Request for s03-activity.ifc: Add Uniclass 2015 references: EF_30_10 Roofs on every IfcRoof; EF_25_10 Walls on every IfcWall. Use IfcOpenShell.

First a look at what the model holds.

```python
import ifcopenshell

model = ifcopenshell.open("s03-activity.ifc")
print(model.schema)
print("classifications:", [c.Name for c in model.by_type("IfcClassification")])
for ifc_class in ("IfcDoor", "IfcRoof", "IfcStair", "IfcWall", "IfcWindow"):
    print(ifc_class, len(model.by_type(ifc_class)))
```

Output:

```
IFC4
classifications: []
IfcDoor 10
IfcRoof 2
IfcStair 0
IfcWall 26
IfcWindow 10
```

```python
import ifcopenshell
import ifcopenshell.api.classification

model = ifcopenshell.open("s03-activity.ifc")

system = ifcopenshell.api.classification.add_classification(model, classification="Uniclass 2015")

codes = {
    "IfcRoof": ("EF_30_10", "Roofs"),
    "IfcWall": ("EF_25_10", "Walls"),
}
for ifc_class, (code, name) in codes.items():
    products = model.by_type(ifc_class)
    ifcopenshell.api.classification.add_reference(
        model, products=products, classification=system, identification=code, name=name
    )
    print(code, len(products))

model.write("s03-activity_v2.ifc")
```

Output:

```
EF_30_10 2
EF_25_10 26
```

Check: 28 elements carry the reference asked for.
